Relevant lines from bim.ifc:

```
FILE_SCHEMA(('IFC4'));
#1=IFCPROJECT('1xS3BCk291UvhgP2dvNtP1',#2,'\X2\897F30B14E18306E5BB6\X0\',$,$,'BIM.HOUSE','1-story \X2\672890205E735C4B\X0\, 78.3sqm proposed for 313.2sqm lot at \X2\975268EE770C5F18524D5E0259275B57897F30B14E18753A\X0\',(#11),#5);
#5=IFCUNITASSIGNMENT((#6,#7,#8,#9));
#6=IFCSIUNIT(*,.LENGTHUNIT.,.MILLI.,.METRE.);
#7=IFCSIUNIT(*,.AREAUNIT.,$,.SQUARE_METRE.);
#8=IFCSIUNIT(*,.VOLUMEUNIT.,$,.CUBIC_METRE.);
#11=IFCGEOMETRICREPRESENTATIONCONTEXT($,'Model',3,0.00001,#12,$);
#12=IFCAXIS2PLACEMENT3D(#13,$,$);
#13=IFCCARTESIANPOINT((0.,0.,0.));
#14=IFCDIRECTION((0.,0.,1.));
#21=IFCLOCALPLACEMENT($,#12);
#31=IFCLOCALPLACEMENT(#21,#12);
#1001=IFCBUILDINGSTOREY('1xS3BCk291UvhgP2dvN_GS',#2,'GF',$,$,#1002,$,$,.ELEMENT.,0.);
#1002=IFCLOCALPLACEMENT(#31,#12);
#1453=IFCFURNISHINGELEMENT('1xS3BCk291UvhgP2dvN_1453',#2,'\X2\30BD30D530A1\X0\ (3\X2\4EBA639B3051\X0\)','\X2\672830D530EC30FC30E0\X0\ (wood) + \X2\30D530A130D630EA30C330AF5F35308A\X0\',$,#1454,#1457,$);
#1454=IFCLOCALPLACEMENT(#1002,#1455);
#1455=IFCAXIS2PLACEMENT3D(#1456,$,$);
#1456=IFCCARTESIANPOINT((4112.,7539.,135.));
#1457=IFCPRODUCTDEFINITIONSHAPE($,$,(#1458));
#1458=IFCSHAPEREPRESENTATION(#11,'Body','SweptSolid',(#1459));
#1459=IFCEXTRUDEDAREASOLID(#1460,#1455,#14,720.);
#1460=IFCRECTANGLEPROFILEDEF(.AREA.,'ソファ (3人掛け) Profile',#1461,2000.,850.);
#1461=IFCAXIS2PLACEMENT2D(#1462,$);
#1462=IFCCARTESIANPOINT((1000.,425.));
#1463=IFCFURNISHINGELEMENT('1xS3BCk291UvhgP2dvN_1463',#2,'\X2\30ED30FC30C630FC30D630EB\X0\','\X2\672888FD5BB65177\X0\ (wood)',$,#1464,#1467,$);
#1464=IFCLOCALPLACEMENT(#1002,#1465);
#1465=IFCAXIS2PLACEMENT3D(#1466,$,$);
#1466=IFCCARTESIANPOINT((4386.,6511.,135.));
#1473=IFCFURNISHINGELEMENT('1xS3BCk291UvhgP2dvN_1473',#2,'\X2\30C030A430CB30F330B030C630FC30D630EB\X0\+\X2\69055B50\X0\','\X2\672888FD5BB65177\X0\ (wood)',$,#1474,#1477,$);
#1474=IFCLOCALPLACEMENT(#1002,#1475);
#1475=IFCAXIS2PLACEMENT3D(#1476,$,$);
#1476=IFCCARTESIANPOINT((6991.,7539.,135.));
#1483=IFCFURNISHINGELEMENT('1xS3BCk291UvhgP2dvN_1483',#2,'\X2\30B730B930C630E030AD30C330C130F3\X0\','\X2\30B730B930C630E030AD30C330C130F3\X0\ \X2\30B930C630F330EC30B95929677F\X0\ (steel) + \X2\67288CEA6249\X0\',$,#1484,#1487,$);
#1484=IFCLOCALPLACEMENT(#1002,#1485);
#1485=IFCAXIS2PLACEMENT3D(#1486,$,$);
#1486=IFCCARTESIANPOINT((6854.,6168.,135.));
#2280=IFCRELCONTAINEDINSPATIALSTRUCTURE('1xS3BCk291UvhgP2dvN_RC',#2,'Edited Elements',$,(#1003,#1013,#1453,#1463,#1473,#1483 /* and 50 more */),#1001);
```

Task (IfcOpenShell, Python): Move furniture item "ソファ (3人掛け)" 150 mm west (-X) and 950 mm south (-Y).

```python
import ifcopenshell
import ifcopenshell.api.geometry
import ifcopenshell.util.placement
import ifcopenshell.util.unit

model = ifcopenshell.open("bim.ifc")
unit_scale = ifcopenshell.util.unit.calculate_unit_scale(model)

item = model.by_id(1453)
matrix = ifcopenshell.util.placement.get_local_placement(item.ObjectPlacement)
matrix[0, 3] -= 0.15 / unit_scale
matrix[1, 3] -= 0.95 / unit_scale
ifcopenshell.api.geometry.edit_object_placement(model, product=item, matrix=matrix, is_si=False)

print(ifcopenshell.util.placement.get_local_placement(item.ObjectPlacement).round(3) + 0.0)

model.write("bim_edited.ifc")
```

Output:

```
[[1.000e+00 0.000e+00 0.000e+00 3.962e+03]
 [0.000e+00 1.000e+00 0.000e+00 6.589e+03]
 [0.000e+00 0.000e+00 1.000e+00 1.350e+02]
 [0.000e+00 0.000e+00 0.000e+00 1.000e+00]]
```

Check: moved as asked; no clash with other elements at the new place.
